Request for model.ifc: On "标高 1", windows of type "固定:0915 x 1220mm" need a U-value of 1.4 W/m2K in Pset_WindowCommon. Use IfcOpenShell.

First a look at what the model holds.

```python
import ifcopenshell
import ifcopenshell.util.element

model = ifcopenshell.open("model.ifc")
print(model.schema)
storey = next(s for s in model.by_type("IfcBuildingStorey") if s.Name == "标高 1")
windows = [e for e in ifcopenshell.util.element.get_decomposition(storey) if e.is_a("IfcWindow")]
seen = {}
for e in windows:
    element_type = ifcopenshell.util.element.get_type(e)
    key = (element_type.Name if element_type != e and element_type else None, ifcopenshell.util.element.get_pset(e, "Pset_WindowCommon", "ThermalTransmittance"))
    seen[key] = seen.get(key, 0) + 1
for (name, value), count in sorted(seen.items(), key=str):
    print(count, "x", name, "|", value)
```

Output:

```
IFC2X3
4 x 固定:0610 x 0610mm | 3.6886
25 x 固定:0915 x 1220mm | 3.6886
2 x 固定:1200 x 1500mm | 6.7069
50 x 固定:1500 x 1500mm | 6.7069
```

```python
import ifcopenshell
import ifcopenshell.api.pset
import ifcopenshell.util.element

model = ifcopenshell.open("model.ifc")

storey = next(s for s in model.by_type("IfcBuildingStorey") if s.Name == "标高 1")
windows = [e for e in ifcopenshell.util.element.get_decomposition(storey) if e.is_a("IfcWindow")]

count = 0
for e in windows:
    element_type = ifcopenshell.util.element.get_type(e)
    if element_type in (None, e) or element_type.Name != "固定:0915 x 1220mm":
        continue
    # add_pset returns the element's existing set when there is one.
    pset = ifcopenshell.api.pset.add_pset(model, product=e, name="Pset_WindowCommon")
    ifcopenshell.api.pset.edit_pset(model, pset=pset, properties={"ThermalTransmittance": 1.4})
    count += 1

print(count, "windows updated")

model.write("model_rev.ifc")
```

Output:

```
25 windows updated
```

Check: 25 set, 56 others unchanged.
